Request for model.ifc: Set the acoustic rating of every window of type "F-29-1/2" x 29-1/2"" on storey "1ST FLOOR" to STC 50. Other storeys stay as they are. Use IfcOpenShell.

First a look at what the model holds.

```python
import ifcopenshell
import ifcopenshell.util.element

model = ifcopenshell.open("model.ifc")
print(model.schema)
storey = next(s for s in model.by_type("IfcBuildingStorey") if s.Name == "1ST FLOOR")
windows = [e for e in ifcopenshell.util.element.get_decomposition(storey) if e.is_a("IfcWindow")]
seen = {}
for e in windows:
    element_type = ifcopenshell.util.element.get_type(e)
    key = (element_type.Name if element_type != e and element_type else None, ifcopenshell.util.element.get_pset(e, "Pset_WindowCommon", "AcousticRating"))
    seen[key] = seen.get(key, 0) + 1
for (name, value), count in sorted(seen.items(), key=str):
    print(count, "x", name, "|", value)
```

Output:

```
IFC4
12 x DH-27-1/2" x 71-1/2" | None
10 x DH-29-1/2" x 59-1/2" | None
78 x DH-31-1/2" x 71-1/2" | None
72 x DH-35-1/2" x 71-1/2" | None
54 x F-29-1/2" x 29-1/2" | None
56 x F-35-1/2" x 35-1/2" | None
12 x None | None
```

```python
import ifcopenshell
import ifcopenshell.api.pset
import ifcopenshell.util.element

model = ifcopenshell.open("model.ifc")

storey = next(s for s in model.by_type("IfcBuildingStorey") if s.Name == "1ST FLOOR")
windows = [e for e in ifcopenshell.util.element.get_decomposition(storey) if e.is_a("IfcWindow")]

count = 0
for e in windows:
    element_type = ifcopenshell.util.element.get_type(e)
    if element_type in (None, e) or element_type.Name != 'F-29-1/2" x 29-1/2"':
        continue
    # add_pset returns the element's existing set when there is one.
    pset = ifcopenshell.api.pset.add_pset(model, product=e, name="Pset_WindowCommon")
    ifcopenshell.api.pset.edit_pset(model, pset=pset, properties={"AcousticRating": "STC 50"})
    count += 1

print(count, "windows updated")

model.write("model_rev.ifc")
```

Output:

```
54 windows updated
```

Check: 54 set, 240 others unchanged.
